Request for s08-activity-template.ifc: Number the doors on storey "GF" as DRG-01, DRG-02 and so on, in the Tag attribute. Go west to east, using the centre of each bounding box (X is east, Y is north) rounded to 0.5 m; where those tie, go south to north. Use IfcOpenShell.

First a look at what the model holds.

```python
import ifcopenshell
import ifcopenshell.util.element
import ifcopenshell.util.placement

model = ifcopenshell.open("s08-activity-template.ifc")
print(model.schema)
storey = next(s for s in model.by_type("IfcBuildingStorey") if s.Name == "GF")
doors = [e for e in ifcopenshell.util.element.get_decomposition(storey) if e.is_a("IfcDoor")]
for e in sorted(doors, key=lambda e: e.id()):
    origin = ifcopenshell.util.placement.get_local_placement(e.ObjectPlacement)[:3, 3]
    print(e.id(), e.Tag, e.Name, origin.round(2) + 0.0, sep=" | ")
```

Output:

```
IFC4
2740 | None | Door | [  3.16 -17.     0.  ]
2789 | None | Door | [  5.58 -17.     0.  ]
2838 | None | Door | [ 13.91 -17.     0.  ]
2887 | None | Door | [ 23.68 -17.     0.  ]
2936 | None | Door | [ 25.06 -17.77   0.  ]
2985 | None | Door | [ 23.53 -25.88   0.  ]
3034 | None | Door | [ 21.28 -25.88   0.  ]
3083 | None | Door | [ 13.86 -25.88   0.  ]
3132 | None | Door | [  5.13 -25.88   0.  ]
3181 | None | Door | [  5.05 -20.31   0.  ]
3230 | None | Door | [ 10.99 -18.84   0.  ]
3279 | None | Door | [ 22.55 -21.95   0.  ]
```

```python
import ifcopenshell
import ifcopenshell.geom
import ifcopenshell.util.element
import ifcopenshell.util.shape

model = ifcopenshell.open("s08-activity-template.ifc")
settings = ifcopenshell.geom.settings()
settings.set("use-world-coords", True)


def centre(element):
    shape = ifcopenshell.geom.create_shape(settings, element)
    return ifcopenshell.util.shape.get_bbox_centroid(shape.geometry)


storey = next(s for s in model.by_type("IfcBuildingStorey") if s.Name == "GF")
doors = [e for e in ifcopenshell.util.element.get_decomposition(storey) if e.is_a("IfcDoor")]

# Insertion points can sit at a corner or the storey origin, so sort by the geometry (in metres).
centres = {e: centre(e) for e in doors}
doors.sort(key=lambda e: (round(centres[e][0] / 0.5), centres[e][1]))

for i, e in enumerate(doors, start=1):
    number = f"DRG-{i:02d}"
    e.Tag = number
    print(e.id(), number)

model.write("s08-activity-template_rev.ifc")
```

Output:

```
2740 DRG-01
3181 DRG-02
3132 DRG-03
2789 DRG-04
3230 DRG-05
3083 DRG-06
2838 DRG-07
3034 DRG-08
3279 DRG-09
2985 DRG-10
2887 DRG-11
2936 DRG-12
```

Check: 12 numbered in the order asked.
